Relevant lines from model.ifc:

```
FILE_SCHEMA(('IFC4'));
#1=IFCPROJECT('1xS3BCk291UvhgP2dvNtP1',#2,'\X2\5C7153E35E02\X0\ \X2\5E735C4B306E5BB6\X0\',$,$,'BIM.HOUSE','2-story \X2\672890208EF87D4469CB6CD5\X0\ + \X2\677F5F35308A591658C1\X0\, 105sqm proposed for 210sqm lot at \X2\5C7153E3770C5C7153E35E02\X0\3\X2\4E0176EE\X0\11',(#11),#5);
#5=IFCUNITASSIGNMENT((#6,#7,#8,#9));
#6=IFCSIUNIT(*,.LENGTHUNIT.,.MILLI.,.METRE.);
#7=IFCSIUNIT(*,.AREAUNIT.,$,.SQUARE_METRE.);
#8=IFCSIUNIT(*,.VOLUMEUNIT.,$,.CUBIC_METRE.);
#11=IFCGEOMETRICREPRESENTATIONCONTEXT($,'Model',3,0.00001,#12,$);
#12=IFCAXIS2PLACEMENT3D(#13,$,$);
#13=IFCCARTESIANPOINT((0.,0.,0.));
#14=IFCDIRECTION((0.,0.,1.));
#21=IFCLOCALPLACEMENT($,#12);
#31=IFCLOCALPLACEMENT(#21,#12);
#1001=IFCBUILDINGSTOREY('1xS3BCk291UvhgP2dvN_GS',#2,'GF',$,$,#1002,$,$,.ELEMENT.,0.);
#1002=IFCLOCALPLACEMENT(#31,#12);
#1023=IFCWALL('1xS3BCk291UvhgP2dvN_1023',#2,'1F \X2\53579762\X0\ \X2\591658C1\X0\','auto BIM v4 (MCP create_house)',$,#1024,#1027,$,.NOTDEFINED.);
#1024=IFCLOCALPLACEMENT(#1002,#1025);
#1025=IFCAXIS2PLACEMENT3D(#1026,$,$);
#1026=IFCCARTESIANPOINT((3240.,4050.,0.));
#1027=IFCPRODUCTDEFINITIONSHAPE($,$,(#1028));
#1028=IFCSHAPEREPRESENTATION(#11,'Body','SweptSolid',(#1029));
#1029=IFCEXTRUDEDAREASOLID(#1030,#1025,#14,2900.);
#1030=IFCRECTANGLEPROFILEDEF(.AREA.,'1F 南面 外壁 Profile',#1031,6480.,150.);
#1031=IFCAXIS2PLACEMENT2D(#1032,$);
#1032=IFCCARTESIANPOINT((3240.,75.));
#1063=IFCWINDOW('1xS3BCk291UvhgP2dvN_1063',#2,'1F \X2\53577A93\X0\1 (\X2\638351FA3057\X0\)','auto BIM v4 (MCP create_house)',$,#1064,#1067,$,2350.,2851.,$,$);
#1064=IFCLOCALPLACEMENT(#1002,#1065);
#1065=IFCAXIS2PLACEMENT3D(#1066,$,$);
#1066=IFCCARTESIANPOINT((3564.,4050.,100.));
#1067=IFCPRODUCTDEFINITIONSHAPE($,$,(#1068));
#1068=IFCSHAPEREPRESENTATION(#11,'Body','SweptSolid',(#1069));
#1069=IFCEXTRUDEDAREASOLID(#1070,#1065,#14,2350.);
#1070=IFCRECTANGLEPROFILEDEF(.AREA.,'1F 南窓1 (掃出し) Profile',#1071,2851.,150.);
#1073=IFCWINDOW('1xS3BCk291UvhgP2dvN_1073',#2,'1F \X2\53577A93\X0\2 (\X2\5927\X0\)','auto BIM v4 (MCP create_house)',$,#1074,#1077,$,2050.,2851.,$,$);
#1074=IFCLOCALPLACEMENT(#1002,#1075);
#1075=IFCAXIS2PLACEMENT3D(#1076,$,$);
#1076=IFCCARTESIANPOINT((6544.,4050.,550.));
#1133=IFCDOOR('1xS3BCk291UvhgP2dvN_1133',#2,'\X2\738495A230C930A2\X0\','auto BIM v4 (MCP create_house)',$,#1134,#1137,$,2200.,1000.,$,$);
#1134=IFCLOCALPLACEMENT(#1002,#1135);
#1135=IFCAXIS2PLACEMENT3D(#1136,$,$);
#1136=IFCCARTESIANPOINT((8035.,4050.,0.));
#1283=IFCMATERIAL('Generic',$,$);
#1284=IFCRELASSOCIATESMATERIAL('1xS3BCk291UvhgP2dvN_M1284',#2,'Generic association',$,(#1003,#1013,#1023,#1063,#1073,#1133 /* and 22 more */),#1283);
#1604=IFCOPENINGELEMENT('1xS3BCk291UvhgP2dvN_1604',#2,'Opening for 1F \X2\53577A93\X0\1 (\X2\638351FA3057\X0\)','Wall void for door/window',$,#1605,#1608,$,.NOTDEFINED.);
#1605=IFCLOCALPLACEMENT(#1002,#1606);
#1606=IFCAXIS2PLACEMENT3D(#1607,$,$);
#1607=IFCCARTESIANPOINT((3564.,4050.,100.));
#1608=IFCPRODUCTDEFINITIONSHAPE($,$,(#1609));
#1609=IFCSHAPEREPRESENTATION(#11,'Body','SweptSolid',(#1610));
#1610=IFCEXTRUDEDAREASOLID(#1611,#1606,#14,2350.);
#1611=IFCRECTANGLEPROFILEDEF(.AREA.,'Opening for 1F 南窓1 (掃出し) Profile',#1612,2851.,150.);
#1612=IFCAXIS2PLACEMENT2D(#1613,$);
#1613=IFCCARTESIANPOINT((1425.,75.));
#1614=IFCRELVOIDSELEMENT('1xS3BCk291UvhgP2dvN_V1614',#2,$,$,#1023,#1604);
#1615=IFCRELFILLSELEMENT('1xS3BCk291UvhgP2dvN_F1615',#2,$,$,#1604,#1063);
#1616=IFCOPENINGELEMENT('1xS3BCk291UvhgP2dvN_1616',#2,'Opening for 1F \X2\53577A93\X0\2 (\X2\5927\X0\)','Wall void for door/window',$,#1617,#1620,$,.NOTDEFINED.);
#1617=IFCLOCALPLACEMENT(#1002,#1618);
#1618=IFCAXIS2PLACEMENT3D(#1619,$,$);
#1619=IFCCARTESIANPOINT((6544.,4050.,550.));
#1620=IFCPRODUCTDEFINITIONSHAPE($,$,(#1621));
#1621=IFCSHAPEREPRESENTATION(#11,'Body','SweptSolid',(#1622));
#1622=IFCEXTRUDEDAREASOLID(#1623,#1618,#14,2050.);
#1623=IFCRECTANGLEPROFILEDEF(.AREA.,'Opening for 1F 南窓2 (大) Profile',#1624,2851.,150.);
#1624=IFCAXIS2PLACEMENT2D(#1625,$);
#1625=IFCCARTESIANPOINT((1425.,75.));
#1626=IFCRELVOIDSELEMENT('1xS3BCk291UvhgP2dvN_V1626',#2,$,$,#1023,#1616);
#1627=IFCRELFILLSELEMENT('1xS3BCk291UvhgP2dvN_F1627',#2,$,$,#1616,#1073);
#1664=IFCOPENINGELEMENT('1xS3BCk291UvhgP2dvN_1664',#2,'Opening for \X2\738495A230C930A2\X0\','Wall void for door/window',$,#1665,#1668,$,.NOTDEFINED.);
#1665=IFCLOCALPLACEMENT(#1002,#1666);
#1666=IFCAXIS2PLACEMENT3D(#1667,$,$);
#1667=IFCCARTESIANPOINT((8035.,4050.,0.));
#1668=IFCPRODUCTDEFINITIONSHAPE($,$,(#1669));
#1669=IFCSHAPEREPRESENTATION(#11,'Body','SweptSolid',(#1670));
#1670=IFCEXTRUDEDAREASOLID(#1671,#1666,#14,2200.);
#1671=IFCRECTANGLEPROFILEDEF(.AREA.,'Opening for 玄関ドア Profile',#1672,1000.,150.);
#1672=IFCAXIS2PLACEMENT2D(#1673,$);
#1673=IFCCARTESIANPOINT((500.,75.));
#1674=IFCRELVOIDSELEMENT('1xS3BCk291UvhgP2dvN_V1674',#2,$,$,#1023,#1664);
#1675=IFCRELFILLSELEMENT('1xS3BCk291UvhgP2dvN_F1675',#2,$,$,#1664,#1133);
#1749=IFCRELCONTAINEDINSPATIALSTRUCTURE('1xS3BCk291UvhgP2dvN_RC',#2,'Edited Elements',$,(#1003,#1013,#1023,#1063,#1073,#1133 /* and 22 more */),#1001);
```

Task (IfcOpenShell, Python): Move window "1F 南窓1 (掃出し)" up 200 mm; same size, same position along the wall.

```python
import numpy as np
import ifcopenshell
import ifcopenshell.api.geometry
import ifcopenshell.util.placement
import ifcopenshell.util.unit

model = ifcopenshell.open("model.ifc")
unit_scale = ifcopenshell.util.unit.calculate_unit_scale(model)

window = model.by_id(1063)
opening = window.FillsVoids[0].RelatingOpeningElement
dz = 0.2 / unit_scale

shift = np.array([0.0, 0.0, dz])
# The window is not placed relative to its opening, so move both.
for product in (opening, window):
    matrix = ifcopenshell.util.placement.get_local_placement(product.ObjectPlacement)
    matrix[:3, 3] += shift
    ifcopenshell.api.geometry.edit_object_placement(model, product=product, matrix=matrix, is_si=False)

print(f"moved by {dz * unit_scale:+.3f} m")

model.write("model_updated.ifc")
```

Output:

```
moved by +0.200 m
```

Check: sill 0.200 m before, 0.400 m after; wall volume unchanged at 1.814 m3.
